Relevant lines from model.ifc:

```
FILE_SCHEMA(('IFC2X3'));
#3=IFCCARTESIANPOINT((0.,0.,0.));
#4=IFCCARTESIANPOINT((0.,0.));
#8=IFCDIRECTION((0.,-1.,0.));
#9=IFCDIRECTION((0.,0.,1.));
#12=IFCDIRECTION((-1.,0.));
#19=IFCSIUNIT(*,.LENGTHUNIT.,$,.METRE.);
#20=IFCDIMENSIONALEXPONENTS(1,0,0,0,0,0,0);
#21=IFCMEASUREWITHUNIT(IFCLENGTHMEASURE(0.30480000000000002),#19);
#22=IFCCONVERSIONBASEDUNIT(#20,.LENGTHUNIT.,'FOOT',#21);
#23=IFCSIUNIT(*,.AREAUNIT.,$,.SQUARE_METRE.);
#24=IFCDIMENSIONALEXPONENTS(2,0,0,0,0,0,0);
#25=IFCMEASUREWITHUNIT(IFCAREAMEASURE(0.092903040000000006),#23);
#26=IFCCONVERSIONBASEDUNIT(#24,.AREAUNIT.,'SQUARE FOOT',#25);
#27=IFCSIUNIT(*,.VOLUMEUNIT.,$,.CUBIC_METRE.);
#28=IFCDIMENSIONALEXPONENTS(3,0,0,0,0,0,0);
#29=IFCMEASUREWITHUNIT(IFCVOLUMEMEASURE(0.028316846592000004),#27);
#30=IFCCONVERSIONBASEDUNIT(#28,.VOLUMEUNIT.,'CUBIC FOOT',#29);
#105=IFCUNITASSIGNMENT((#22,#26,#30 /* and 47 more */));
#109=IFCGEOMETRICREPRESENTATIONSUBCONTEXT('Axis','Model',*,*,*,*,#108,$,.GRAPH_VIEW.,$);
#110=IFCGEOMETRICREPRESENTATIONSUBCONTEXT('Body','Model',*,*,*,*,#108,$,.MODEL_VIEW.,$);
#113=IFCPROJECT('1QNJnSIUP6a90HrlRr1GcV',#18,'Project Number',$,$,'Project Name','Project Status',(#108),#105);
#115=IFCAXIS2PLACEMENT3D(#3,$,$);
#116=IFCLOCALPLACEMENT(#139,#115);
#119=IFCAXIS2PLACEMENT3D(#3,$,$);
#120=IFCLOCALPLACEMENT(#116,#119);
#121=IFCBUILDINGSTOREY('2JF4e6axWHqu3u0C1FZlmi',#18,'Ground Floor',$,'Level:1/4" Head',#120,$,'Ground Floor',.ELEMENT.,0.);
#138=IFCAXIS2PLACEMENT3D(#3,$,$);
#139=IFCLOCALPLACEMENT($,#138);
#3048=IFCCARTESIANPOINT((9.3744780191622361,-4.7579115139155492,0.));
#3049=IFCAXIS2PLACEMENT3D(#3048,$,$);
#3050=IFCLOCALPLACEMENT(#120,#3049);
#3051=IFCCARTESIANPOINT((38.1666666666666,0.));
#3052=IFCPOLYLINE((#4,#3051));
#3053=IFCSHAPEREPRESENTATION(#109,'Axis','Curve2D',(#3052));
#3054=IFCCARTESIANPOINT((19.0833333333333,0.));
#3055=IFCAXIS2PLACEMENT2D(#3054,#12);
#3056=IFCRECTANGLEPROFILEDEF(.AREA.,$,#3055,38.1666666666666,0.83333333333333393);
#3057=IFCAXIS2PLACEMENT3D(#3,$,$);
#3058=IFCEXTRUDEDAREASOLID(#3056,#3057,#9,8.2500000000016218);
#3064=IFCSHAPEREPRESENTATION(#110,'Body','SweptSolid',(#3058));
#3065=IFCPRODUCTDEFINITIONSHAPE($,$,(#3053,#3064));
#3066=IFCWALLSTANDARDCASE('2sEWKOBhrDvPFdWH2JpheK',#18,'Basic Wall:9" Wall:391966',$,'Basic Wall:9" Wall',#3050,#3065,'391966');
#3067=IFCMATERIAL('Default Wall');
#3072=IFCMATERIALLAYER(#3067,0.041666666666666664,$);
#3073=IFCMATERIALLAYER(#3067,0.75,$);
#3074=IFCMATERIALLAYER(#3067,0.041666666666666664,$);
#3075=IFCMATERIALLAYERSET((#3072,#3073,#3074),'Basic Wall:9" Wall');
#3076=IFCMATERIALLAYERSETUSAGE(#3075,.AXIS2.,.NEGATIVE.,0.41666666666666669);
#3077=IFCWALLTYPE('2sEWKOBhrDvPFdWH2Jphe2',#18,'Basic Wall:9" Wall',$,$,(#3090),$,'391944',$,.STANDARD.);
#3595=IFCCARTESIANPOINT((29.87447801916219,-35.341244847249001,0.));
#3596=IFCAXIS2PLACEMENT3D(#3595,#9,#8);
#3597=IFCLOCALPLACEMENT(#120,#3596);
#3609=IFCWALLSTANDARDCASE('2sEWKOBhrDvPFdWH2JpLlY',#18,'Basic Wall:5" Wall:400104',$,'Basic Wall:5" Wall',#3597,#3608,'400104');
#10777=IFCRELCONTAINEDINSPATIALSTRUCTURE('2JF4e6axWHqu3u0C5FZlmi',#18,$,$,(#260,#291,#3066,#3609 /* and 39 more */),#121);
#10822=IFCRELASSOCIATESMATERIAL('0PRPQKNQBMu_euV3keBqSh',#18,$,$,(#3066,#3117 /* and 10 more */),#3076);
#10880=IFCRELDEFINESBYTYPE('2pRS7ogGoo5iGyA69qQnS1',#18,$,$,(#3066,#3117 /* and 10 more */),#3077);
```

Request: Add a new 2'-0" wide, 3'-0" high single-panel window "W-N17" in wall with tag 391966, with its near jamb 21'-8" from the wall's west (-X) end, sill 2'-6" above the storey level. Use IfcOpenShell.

```python
import numpy as np
import ifcopenshell
import ifcopenshell.api.feature
import ifcopenshell.api.geometry
import ifcopenshell.api.root
import ifcopenshell.api.spatial
import ifcopenshell.api.type
import ifcopenshell.geom
import ifcopenshell.util.element
import ifcopenshell.util.placement
import ifcopenshell.util.representation
import ifcopenshell.util.shape
import ifcopenshell.util.unit

model = ifcopenshell.open("model.ifc")
unit_scale = ifcopenshell.util.unit.calculate_unit_scale(model)
settings = ifcopenshell.geom.settings()


def volume(element):
    """Net volume in cubic metres, openings subtracted."""
    shape = ifcopenshell.geom.create_shape(settings, element)
    return ifcopenshell.util.shape.get_volume(shape.geometry)


wall = model.by_guid("2sEWKOBhrDvPFdWH2JpheK")
storey = ifcopenshell.util.element.get_container(wall, ifc_class="IfcBuildingStorey")
context = ifcopenshell.util.representation.get_context(model, "Model", "Body", "MODEL_VIEW")
before = volume(wall)

width, height, from_end, sill = 0.6096, 0.9144, 6.604, 0.762  # metres

# The wall runs along its own X axis, and the end named is its -X end.
wall_shape = ifcopenshell.geom.create_shape(settings, wall)
x, y, z = ifcopenshell.util.shape.get_vertices(wall_shape.geometry).T
start = x.min() + from_end
face, thickness = float(y.min()), float(y.max() - y.min())
wall_matrix = ifcopenshell.util.placement.get_local_placement(wall.ObjectPlacement)
level = ifcopenshell.util.placement.get_local_placement(storey.ObjectPlacement)[2, 3]


def in_wall(x, y):
    """Placement at x, y metres in the wall's axes, at sill height."""
    matrix = wall_matrix.copy()
    matrix[:, 3] = wall_matrix @ np.array([x / unit_scale, y / unit_scale, 0.0, 1.0])
    matrix[2, 3] = level + sill / unit_scale
    return matrix


# Opening: a box that overshoots both wall faces by 50 mm.
opening = ifcopenshell.api.root.create_entity(model, ifc_class="IfcOpeningElement")
box = ifcopenshell.api.geometry.add_wall_representation(
    model, context=context, length=width, height=height, thickness=thickness + 0.1
)
ifcopenshell.api.geometry.assign_representation(model, product=opening, representation=box)
ifcopenshell.api.geometry.edit_object_placement(model, product=opening, matrix=in_wall(start, face - 0.05), is_si=False)
ifcopenshell.api.feature.add_feature(model, feature=opening, element=wall)

window = ifcopenshell.api.root.create_entity(model, ifc_class="IfcWindow", name="W-N17")
window.OverallWidth, window.OverallHeight = width / unit_scale, height / unit_scale
body = ifcopenshell.api.geometry.add_window_representation(
    model,
    context=context,
    overall_width=window.OverallWidth,
    overall_height=window.OverallHeight,
    partition_type="SINGLE_PANEL",
)
ifcopenshell.api.geometry.assign_representation(model, product=window, representation=body)
ifcopenshell.api.spatial.assign_container(model, products=[window], relating_structure=storey)
fills = ifcopenshell.api.feature.add_filling(model, opening=opening, element=window)
fills.OwnerHistory = window.OwnerHistory  # required in IFC2X3

# IFC2X3 keeps the operation on the window style.
style = ifcopenshell.api.root.create_entity(model, ifc_class="IfcWindowStyle", name="W-N17")
style.OperationType, style.ConstructionType = "SINGLE_PANEL", "NOTDEFINED"
style.ParameterTakesPrecedence = style.Sizeable = False
ifcopenshell.api.type.assign_type(model, related_objects=[window], relating_type=style)

# Centre the window in the wall's thickness.
ifcopenshell.api.geometry.edit_object_placement(model, product=window, matrix=in_wall(start, face), is_si=False)
window_shape = ifcopenshell.geom.create_shape(settings, window)
depth = ifcopenshell.util.shape.get_vertices(window_shape.geometry)[:, 1]
offset = face + thickness / 2 - (depth.min() + depth.max()) / 2
ifcopenshell.api.geometry.edit_object_placement(model, product=window, matrix=in_wall(start, offset), is_si=False)

after = volume(wall)

print(f"wall volume {before:.3f} -> {after:.3f} m3")

model.write("model_updated.ifc")
```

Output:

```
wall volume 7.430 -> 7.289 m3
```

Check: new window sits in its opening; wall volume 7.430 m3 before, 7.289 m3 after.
